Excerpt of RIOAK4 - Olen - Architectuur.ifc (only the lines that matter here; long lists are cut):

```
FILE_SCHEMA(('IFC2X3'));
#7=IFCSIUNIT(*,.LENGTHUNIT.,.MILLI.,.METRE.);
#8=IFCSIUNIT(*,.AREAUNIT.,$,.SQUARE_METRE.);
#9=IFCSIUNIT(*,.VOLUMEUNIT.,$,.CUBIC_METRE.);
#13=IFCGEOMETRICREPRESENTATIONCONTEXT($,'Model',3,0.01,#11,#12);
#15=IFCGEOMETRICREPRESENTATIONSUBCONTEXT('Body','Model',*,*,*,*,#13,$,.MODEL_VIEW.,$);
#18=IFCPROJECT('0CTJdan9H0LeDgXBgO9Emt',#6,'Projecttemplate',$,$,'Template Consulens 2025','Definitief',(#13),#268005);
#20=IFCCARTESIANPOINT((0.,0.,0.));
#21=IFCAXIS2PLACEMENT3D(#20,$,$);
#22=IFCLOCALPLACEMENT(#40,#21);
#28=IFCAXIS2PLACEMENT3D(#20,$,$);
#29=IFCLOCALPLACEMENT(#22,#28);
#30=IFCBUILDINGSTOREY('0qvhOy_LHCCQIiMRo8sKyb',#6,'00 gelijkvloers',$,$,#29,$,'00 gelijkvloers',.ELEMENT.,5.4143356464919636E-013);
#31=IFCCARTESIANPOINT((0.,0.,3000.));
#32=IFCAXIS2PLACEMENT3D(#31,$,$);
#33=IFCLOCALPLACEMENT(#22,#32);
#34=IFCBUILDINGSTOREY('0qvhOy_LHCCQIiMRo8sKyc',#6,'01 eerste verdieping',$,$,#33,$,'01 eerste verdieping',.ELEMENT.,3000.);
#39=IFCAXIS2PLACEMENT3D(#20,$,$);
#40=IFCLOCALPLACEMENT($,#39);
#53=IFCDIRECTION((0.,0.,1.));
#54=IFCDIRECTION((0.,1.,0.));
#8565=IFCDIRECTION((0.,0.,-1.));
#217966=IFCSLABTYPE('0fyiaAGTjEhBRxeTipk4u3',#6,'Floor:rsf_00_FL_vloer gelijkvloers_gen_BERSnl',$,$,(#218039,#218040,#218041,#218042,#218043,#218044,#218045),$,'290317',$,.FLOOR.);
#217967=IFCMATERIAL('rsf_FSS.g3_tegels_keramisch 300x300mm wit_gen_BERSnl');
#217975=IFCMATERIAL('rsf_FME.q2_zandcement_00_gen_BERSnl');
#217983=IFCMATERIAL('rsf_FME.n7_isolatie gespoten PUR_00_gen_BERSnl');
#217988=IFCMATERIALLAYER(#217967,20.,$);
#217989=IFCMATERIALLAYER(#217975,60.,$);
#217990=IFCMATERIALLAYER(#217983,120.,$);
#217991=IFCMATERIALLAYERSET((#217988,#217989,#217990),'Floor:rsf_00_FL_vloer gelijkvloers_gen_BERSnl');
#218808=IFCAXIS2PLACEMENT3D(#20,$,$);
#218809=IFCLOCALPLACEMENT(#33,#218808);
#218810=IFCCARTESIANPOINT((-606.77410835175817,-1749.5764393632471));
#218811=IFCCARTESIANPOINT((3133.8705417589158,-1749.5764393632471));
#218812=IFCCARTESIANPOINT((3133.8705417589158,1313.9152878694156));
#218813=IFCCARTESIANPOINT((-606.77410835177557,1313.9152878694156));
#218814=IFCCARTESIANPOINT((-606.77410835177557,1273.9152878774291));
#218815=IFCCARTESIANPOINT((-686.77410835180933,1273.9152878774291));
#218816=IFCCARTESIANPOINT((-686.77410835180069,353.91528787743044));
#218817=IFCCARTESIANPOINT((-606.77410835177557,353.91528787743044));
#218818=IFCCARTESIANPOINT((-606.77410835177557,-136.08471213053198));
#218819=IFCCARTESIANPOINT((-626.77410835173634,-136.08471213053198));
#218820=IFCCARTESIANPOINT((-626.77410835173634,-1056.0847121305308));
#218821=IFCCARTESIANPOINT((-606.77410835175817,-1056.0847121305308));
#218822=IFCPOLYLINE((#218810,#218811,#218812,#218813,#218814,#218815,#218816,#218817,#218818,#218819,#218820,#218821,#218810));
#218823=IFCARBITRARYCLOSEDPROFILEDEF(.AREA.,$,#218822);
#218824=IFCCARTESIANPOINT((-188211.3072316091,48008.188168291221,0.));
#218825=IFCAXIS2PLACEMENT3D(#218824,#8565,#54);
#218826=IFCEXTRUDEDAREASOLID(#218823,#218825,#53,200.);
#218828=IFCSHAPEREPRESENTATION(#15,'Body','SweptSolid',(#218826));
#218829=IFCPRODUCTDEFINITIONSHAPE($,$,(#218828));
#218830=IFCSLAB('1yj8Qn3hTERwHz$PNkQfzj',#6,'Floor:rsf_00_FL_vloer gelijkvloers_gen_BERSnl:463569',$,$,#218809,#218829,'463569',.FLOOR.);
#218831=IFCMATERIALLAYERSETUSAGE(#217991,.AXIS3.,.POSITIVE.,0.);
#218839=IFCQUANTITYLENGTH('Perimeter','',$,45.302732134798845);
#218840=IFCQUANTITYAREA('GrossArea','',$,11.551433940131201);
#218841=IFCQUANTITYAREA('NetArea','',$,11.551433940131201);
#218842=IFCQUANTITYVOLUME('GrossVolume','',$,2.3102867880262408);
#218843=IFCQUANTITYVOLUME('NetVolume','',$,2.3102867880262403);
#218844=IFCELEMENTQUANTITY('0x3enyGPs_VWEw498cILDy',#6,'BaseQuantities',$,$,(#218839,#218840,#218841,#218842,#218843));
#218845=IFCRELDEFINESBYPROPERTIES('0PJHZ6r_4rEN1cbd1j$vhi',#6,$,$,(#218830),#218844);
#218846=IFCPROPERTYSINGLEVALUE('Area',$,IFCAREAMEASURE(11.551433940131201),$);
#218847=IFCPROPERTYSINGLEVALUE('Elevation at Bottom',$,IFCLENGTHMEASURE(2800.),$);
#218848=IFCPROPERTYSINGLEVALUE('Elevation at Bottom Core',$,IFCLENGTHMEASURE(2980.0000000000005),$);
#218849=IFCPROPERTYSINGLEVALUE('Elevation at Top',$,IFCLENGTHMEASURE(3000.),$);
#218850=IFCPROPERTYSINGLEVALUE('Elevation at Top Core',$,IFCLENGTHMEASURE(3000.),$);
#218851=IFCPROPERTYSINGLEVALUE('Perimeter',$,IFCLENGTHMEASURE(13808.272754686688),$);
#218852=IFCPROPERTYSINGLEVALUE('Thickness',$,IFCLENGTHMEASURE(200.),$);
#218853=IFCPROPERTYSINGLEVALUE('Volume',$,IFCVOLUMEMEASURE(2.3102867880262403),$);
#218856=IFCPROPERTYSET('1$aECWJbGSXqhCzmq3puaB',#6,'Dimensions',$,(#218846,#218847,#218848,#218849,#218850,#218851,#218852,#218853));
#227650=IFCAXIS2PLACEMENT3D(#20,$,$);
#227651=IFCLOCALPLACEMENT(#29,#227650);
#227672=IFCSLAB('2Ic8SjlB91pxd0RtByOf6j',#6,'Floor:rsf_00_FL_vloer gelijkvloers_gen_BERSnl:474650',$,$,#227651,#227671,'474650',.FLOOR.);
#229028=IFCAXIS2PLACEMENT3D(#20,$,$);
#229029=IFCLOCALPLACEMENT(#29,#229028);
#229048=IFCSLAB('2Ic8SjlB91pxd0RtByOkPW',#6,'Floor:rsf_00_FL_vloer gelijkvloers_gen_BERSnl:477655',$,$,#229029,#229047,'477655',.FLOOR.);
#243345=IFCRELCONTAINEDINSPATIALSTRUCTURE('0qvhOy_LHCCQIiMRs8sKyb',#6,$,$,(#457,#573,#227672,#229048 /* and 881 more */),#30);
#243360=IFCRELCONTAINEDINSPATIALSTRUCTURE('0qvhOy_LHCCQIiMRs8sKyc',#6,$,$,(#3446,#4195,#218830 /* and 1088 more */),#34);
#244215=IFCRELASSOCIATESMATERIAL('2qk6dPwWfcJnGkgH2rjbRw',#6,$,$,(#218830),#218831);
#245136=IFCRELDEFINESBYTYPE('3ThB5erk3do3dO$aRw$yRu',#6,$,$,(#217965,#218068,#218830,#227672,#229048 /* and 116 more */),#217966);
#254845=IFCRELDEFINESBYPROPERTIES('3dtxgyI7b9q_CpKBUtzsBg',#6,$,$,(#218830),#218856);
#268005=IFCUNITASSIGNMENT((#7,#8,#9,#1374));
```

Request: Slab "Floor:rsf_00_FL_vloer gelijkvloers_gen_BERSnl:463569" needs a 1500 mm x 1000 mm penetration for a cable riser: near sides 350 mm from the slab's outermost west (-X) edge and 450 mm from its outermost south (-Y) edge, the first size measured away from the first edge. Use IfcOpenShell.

```python
import numpy as np
import ifcopenshell
import ifcopenshell.api.feature
import ifcopenshell.api.geometry
import ifcopenshell.api.pset
import ifcopenshell.api.root
import ifcopenshell.geom
import ifcopenshell.util.element
import ifcopenshell.util.placement
import ifcopenshell.util.representation
import ifcopenshell.util.shape
import ifcopenshell.util.unit

model = ifcopenshell.open("RIOAK4 - Olen - Architectuur.ifc")
unit_scale = ifcopenshell.util.unit.calculate_unit_scale(model)
area_scale = ifcopenshell.util.unit.calculate_unit_scale(model, "AREAUNIT")
volume_scale = ifcopenshell.util.unit.calculate_unit_scale(model, "VOLUMEUNIT")
settings = ifcopenshell.geom.settings()


def volume(element):
    """Net volume in cubic metres, openings subtracted."""
    shape = ifcopenshell.geom.create_shape(settings, element)
    return ifcopenshell.util.shape.get_volume(shape.geometry)


slab = model.by_id(218830)
before = volume(slab)

# Extent in the slab's own axes, in metres. The edges named are its -X and -Y sides.
slab_shape = ifcopenshell.geom.create_shape(settings, slab)
vertices = ifcopenshell.util.shape.get_vertices(slab_shape.geometry)
x_min, y_min, bottom = vertices.min(axis=0)
top = vertices[:, 2].max()

opening = ifcopenshell.api.root.create_entity(model, ifc_class="IfcOpeningElement", name="Cable riser opening")
context = ifcopenshell.util.representation.get_context(model, "Model", "Body", "MODEL_VIEW")
width, depth = 1.5, 1
outline = [(0.0, 0.0), (width, 0.0), (width, depth), (0.0, depth), (0.0, 0.0)]
# Overshoot both faces by 50 mm so the cut is clean.
shape = ifcopenshell.api.geometry.add_slab_representation(
    model, context=context, depth=top - bottom + 0.1, polyline=outline
)
ifcopenshell.api.geometry.assign_representation(model, product=opening, representation=shape)

matrix = ifcopenshell.util.placement.get_local_placement(slab.ObjectPlacement)
matrix[:, 3] = matrix @ np.append(np.array([x_min + 0.35, y_min + 0.45, bottom - 0.05]) / unit_scale, 1.0)
ifcopenshell.api.geometry.edit_object_placement(model, product=opening, matrix=matrix, is_si=False)
ifcopenshell.api.feature.add_feature(model, feature=opening, element=slab)

after = volume(slab)

# Update the slab's stored quantities.
qto = model.by_id(ifcopenshell.util.element.get_pset(slab, "BaseQuantities", should_inherit=False)["id"])
ifcopenshell.api.pset.edit_qto(model, qto=qto, properties={
    "NetArea": after / (top - bottom) / area_scale,
    "NetVolume": after / volume_scale,
})
pset = model.by_id(ifcopenshell.util.element.get_pset(slab, "Dimensions", should_inherit=False)["id"])
ifcopenshell.api.pset.edit_pset(model, pset=pset, properties={
    "Area": model.create_entity("IfcAreaMeasure", after / (top - bottom) / area_scale),
    "Volume": model.create_entity("IfcVolumeMeasure", after / volume_scale),
})

print(f"slab volume {before:.3f} -> {after:.3f} m3")

model.write("RIOAK4 - Olen - Architectuur_edited.ifc")
```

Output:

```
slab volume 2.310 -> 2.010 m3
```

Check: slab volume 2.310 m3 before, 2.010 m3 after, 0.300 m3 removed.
